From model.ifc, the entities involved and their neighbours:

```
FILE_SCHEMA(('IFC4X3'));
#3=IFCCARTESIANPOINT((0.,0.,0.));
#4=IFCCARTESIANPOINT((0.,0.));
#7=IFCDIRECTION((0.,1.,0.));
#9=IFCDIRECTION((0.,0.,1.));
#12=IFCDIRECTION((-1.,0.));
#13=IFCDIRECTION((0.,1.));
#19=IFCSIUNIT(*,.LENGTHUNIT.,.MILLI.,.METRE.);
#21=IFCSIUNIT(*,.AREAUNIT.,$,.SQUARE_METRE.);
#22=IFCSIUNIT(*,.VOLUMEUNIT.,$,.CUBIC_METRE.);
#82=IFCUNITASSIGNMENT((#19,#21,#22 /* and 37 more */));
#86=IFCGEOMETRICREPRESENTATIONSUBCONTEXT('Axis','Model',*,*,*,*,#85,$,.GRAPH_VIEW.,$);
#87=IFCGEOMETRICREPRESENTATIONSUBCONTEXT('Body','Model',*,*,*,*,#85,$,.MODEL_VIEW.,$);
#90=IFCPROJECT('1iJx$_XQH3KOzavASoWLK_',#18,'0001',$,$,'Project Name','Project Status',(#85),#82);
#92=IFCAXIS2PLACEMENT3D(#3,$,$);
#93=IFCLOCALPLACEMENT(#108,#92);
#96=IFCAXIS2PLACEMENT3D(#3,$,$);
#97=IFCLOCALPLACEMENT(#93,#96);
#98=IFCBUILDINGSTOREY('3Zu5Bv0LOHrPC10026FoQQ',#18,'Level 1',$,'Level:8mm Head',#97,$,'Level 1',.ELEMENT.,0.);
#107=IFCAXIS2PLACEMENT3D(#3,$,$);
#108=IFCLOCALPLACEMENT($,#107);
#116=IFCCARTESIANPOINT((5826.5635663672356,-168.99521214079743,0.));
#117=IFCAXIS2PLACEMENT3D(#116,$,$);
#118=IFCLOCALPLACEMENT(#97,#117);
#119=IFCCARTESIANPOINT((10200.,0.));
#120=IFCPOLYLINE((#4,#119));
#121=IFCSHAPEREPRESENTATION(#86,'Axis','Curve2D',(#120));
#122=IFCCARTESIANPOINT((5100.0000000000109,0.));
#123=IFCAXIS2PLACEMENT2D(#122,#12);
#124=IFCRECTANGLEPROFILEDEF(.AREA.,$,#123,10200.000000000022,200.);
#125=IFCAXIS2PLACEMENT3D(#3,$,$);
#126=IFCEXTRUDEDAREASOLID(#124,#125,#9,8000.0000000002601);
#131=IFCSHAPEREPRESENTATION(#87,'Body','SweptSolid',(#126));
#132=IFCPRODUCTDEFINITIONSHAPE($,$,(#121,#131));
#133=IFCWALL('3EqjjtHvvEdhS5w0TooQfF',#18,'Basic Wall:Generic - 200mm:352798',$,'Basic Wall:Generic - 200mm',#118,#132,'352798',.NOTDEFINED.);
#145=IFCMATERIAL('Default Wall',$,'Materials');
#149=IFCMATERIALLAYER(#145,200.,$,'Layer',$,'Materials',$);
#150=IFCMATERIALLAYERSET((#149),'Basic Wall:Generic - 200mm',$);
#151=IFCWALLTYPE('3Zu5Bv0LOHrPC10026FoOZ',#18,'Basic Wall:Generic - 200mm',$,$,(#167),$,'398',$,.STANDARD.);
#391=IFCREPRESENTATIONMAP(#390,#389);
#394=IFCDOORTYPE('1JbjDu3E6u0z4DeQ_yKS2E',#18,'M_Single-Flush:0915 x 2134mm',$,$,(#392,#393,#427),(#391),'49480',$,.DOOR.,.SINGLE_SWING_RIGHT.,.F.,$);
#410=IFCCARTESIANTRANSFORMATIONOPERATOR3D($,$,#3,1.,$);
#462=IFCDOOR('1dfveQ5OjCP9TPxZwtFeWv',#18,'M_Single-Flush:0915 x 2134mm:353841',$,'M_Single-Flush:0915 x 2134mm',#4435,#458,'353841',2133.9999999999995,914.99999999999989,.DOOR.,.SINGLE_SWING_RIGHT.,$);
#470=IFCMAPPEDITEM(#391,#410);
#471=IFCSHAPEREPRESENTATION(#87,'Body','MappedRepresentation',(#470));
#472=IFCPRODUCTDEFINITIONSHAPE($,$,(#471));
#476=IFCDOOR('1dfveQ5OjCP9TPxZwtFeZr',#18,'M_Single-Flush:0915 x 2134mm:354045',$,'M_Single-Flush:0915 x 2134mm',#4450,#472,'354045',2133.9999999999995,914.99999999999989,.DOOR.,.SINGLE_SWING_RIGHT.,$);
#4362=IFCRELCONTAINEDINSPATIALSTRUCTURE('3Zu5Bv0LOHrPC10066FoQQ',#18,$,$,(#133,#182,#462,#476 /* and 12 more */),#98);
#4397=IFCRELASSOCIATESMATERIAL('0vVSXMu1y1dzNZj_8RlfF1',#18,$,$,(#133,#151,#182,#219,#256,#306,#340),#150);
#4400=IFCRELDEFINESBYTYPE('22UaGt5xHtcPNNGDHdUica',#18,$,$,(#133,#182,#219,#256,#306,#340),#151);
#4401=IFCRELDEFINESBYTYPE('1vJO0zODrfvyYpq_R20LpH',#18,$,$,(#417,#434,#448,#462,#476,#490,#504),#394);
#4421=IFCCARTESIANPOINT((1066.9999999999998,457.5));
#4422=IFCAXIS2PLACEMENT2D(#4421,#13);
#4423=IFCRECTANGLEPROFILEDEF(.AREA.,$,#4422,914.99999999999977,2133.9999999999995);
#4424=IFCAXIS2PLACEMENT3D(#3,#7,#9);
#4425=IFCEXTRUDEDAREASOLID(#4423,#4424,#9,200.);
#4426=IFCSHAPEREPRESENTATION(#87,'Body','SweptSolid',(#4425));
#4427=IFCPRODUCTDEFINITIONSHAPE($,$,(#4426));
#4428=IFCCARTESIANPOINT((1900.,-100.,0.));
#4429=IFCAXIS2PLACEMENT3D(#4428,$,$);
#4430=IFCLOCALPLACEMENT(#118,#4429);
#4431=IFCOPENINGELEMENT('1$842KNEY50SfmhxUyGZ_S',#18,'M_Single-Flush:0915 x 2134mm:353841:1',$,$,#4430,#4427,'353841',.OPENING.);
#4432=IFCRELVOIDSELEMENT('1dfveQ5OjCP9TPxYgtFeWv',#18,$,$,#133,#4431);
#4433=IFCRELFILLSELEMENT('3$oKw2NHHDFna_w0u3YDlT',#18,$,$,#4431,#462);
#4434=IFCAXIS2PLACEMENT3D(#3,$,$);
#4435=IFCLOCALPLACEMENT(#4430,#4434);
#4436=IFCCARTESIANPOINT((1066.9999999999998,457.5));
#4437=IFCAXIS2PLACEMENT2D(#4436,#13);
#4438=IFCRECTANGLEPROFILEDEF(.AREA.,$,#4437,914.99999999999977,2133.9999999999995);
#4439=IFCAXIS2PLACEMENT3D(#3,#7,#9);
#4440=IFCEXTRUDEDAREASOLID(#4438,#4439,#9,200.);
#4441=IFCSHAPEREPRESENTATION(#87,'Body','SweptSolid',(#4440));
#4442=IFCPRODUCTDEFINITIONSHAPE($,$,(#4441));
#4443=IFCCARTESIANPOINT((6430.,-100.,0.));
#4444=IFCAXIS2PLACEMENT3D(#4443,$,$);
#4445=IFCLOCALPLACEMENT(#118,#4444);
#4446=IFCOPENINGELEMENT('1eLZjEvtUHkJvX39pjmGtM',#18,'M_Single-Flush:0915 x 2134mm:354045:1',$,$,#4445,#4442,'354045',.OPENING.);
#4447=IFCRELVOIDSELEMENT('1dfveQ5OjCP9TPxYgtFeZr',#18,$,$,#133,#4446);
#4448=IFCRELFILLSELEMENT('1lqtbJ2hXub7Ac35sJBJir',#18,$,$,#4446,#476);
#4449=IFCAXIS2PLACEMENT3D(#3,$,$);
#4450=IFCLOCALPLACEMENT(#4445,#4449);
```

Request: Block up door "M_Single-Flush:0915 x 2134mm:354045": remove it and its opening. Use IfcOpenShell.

```python
import ifcopenshell
import ifcopenshell.api.feature
import ifcopenshell.api.root
import ifcopenshell.geom
import ifcopenshell.util.shape

model = ifcopenshell.open("model.ifc")
settings = ifcopenshell.geom.settings()


def volume(element):
    """Net volume in cubic metres, openings subtracted."""
    shape = ifcopenshell.geom.create_shape(settings, element)
    return ifcopenshell.util.shape.get_volume(shape.geometry)


door = model.by_id(476)
opening = door.FillsVoids[0].RelatingOpeningElement
wall = opening.VoidsElements[0].RelatingBuildingElement
before = volume(wall)

ifcopenshell.api.root.remove_product(model, product=door)
ifcopenshell.api.feature.remove_feature(model, feature=opening)

after = volume(wall)

print(f"wall volume {before:.3f} -> {after:.3f} m3")

model.write("model_edited.ifc")
```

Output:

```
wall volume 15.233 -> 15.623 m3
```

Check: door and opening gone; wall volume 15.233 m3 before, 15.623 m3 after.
